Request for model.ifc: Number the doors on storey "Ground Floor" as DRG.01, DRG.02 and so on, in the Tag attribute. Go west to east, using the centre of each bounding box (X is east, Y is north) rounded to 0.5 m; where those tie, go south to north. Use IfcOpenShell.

First a look at what the model holds.

```python
import ifcopenshell
import ifcopenshell.util.element
import ifcopenshell.util.placement

model = ifcopenshell.open("model.ifc")
print(model.schema)
storey = next(s for s in model.by_type("IfcBuildingStorey") if s.Name == "Ground Floor")
doors = [e for e in ifcopenshell.util.element.get_decomposition(storey) if e.is_a("IfcDoor")]
for e in sorted(doors, key=lambda e: e.id()):
    origin = ifcopenshell.util.placement.get_local_placement(e.ObjectPlacement)[:3, 3]
    print(e.id(), e.Tag, e.Name, origin.round(2) + 0.0, sep=" | ")
```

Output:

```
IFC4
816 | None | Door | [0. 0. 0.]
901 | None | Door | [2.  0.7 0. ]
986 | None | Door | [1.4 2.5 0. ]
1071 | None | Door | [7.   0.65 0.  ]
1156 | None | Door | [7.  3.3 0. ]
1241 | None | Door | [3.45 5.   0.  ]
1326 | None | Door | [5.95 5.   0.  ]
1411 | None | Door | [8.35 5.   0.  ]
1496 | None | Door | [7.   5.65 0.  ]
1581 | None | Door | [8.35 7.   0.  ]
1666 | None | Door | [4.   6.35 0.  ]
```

```python
import ifcopenshell
import ifcopenshell.geom
import ifcopenshell.util.element
import ifcopenshell.util.shape

model = ifcopenshell.open("model.ifc")
settings = ifcopenshell.geom.settings()
settings.set("use-world-coords", True)


def centre(element):
    shape = ifcopenshell.geom.create_shape(settings, element)
    return ifcopenshell.util.shape.get_bbox_centroid(shape.geometry)


storey = next(s for s in model.by_type("IfcBuildingStorey") if s.Name == "Ground Floor")
doors = [e for e in ifcopenshell.util.element.get_decomposition(storey) if e.is_a("IfcDoor")]

# Insertion points can sit at a corner or the storey origin, so sort by the geometry (in metres).
centres = {e: centre(e) for e in doors}
doors.sort(key=lambda e: (round(centres[e][0] / 0.5), centres[e][1]))

for i, e in enumerate(doors, start=1):
    number = f"DRG.{i:02d}"
    e.Tag = number
    print(e.id(), number)

model.write("model-out.ifc")
```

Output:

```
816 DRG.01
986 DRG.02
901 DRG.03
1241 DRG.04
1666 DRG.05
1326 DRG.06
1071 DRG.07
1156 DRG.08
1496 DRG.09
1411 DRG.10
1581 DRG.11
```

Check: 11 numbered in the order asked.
